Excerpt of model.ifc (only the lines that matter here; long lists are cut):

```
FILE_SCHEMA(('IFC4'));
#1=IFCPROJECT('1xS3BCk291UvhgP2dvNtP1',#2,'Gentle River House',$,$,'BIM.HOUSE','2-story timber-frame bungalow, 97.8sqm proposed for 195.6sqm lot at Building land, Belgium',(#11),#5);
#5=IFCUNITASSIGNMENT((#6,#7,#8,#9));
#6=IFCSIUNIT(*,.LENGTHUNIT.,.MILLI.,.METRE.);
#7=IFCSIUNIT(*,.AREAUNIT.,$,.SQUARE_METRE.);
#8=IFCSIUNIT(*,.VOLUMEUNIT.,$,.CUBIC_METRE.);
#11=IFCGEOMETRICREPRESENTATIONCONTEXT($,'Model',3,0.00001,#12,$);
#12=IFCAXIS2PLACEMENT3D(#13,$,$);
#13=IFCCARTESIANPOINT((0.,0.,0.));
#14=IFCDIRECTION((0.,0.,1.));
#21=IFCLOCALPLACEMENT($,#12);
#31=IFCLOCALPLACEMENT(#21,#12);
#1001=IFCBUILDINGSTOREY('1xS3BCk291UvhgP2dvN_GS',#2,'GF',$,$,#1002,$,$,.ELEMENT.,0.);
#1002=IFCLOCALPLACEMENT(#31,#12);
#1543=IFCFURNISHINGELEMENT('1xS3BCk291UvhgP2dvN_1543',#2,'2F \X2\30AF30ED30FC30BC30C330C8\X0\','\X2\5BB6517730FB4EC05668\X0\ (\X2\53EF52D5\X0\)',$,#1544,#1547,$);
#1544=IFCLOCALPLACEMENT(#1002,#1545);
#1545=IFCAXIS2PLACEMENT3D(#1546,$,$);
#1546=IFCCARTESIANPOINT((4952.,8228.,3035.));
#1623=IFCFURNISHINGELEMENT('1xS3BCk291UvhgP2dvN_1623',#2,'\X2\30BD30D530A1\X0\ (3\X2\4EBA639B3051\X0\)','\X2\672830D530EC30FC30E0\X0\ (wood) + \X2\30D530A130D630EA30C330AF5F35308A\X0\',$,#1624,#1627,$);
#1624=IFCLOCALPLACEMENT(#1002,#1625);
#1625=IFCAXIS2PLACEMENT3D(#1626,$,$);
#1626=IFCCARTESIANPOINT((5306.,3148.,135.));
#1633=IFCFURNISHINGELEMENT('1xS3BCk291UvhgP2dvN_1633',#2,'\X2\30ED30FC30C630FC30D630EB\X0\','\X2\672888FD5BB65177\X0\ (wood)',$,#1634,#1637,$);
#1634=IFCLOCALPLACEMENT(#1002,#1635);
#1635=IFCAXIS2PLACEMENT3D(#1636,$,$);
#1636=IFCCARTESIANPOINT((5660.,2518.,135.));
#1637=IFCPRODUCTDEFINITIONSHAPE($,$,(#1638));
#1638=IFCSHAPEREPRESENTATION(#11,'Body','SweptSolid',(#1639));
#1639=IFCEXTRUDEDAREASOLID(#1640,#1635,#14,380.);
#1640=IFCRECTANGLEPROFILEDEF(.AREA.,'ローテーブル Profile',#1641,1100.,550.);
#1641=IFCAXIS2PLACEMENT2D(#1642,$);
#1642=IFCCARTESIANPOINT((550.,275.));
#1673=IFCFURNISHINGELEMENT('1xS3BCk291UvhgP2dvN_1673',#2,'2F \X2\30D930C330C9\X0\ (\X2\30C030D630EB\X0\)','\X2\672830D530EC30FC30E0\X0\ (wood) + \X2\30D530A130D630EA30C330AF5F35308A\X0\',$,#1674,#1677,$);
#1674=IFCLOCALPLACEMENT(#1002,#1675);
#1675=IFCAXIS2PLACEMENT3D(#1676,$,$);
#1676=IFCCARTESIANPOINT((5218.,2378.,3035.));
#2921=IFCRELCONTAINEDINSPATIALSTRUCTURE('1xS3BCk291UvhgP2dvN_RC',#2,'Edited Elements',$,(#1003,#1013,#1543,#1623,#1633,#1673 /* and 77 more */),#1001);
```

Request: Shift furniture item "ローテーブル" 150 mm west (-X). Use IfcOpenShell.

```python
import ifcopenshell
import ifcopenshell.api.geometry
import ifcopenshell.util.placement
import ifcopenshell.util.unit

model = ifcopenshell.open("model.ifc")
unit_scale = ifcopenshell.util.unit.calculate_unit_scale(model)

item = model.by_id(1633)
matrix = ifcopenshell.util.placement.get_local_placement(item.ObjectPlacement)
matrix[0, 3] -= 0.15 / unit_scale
ifcopenshell.api.geometry.edit_object_placement(model, product=item, matrix=matrix, is_si=False)

print(ifcopenshell.util.placement.get_local_placement(item.ObjectPlacement).round(3) + 0.0)

model.write("model_edited.ifc")
```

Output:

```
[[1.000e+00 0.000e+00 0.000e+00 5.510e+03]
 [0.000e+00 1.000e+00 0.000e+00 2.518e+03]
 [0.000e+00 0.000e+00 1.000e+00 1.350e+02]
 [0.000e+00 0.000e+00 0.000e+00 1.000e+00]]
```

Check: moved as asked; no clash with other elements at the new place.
